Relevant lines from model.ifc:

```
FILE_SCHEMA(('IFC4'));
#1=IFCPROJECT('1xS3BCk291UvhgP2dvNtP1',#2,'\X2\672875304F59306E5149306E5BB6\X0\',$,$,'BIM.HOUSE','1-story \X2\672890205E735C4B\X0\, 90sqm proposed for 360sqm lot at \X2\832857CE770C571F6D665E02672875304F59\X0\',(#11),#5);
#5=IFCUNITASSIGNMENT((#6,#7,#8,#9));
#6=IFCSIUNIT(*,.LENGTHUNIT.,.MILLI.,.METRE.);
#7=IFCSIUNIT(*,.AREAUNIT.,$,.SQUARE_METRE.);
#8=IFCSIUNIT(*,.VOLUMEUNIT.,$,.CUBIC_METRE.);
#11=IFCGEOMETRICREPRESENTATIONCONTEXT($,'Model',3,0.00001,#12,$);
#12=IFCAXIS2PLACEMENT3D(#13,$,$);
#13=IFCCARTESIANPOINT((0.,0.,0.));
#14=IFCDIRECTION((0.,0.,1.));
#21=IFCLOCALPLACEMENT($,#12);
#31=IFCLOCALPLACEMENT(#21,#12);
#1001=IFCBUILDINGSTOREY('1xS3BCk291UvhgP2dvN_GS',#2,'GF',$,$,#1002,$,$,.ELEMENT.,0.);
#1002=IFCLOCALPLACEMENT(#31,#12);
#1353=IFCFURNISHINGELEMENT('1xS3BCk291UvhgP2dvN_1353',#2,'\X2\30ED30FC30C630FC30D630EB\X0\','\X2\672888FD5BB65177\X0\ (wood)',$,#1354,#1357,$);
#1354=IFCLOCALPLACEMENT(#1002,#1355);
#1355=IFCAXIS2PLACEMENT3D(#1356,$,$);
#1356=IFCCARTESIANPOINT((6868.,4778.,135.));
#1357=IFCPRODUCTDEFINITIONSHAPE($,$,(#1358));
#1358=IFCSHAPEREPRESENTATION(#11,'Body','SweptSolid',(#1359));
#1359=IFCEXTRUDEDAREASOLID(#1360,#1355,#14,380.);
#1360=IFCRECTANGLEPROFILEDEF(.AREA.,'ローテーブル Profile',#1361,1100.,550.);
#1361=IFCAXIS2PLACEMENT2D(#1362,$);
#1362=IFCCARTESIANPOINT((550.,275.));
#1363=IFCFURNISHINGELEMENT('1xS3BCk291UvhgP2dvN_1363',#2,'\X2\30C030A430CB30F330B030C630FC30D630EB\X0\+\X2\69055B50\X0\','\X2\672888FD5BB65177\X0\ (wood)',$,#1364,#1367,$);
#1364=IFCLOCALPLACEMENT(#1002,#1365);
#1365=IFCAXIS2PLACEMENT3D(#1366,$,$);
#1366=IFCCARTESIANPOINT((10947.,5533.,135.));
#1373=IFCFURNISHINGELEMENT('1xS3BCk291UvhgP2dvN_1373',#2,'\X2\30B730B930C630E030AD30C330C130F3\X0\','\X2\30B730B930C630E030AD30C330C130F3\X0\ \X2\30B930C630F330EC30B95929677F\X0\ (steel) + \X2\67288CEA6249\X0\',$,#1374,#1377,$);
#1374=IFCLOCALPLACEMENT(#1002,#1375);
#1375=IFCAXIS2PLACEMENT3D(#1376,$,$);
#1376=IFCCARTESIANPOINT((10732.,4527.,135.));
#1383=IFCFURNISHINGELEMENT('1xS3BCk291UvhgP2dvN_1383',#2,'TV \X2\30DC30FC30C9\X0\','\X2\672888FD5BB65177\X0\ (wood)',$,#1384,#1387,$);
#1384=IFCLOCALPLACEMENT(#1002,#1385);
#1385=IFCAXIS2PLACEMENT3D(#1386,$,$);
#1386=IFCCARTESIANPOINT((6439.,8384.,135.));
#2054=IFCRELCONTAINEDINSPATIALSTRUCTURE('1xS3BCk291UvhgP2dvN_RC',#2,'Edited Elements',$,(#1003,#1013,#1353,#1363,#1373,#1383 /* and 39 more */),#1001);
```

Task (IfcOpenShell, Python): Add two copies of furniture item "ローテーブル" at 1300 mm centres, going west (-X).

```python
import numpy as np
import ifcopenshell
import ifcopenshell.api.geometry
import ifcopenshell.api.root
import ifcopenshell.util.element
import ifcopenshell.util.placement
import ifcopenshell.util.unit

model = ifcopenshell.open("model.ifc")
unit_scale = ifcopenshell.util.unit.calculate_unit_scale(model)


def reuse_history(source, copy):
    """copy_class also copies each property set's owner history, people and application; keep the originals."""
    for rel in copy.IsDefinedBy:
        if rel.is_a("IfcRelDefinesByProperties") and (history := rel.RelatingPropertyDefinition.OwnerHistory):
            rel.RelatingPropertyDefinition.OwnerHistory = source.OwnerHistory
            ifcopenshell.util.element.remove_deep2(model, history)


source = model.by_guid("1xS3BCk291UvhgP2dvN_1353")
base = ifcopenshell.util.placement.get_local_placement(source.ObjectPlacement)
step = np.array([-1.0, 0.0, 0.0]) * 1.3 / unit_scale

for i in range(1, 3):
    copy = ifcopenshell.api.root.copy_class(model, product=source)
    copy.Representation = ifcopenshell.util.element.copy_deep(
        model, source.Representation, exclude=["IfcGeometricRepresentationContext", "IfcRepresentationMap"]
    )
    reuse_history(source, copy)
    matrix = base.copy()
    matrix[:3, 3] += i * step
    print("added at", matrix[:3, 3].round(3) + 0.0)
    ifcopenshell.api.geometry.edit_object_placement(model, product=copy, matrix=matrix, is_si=False)

model.write("model-out.ifc")
```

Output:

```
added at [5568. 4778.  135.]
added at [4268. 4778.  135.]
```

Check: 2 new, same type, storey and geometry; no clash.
